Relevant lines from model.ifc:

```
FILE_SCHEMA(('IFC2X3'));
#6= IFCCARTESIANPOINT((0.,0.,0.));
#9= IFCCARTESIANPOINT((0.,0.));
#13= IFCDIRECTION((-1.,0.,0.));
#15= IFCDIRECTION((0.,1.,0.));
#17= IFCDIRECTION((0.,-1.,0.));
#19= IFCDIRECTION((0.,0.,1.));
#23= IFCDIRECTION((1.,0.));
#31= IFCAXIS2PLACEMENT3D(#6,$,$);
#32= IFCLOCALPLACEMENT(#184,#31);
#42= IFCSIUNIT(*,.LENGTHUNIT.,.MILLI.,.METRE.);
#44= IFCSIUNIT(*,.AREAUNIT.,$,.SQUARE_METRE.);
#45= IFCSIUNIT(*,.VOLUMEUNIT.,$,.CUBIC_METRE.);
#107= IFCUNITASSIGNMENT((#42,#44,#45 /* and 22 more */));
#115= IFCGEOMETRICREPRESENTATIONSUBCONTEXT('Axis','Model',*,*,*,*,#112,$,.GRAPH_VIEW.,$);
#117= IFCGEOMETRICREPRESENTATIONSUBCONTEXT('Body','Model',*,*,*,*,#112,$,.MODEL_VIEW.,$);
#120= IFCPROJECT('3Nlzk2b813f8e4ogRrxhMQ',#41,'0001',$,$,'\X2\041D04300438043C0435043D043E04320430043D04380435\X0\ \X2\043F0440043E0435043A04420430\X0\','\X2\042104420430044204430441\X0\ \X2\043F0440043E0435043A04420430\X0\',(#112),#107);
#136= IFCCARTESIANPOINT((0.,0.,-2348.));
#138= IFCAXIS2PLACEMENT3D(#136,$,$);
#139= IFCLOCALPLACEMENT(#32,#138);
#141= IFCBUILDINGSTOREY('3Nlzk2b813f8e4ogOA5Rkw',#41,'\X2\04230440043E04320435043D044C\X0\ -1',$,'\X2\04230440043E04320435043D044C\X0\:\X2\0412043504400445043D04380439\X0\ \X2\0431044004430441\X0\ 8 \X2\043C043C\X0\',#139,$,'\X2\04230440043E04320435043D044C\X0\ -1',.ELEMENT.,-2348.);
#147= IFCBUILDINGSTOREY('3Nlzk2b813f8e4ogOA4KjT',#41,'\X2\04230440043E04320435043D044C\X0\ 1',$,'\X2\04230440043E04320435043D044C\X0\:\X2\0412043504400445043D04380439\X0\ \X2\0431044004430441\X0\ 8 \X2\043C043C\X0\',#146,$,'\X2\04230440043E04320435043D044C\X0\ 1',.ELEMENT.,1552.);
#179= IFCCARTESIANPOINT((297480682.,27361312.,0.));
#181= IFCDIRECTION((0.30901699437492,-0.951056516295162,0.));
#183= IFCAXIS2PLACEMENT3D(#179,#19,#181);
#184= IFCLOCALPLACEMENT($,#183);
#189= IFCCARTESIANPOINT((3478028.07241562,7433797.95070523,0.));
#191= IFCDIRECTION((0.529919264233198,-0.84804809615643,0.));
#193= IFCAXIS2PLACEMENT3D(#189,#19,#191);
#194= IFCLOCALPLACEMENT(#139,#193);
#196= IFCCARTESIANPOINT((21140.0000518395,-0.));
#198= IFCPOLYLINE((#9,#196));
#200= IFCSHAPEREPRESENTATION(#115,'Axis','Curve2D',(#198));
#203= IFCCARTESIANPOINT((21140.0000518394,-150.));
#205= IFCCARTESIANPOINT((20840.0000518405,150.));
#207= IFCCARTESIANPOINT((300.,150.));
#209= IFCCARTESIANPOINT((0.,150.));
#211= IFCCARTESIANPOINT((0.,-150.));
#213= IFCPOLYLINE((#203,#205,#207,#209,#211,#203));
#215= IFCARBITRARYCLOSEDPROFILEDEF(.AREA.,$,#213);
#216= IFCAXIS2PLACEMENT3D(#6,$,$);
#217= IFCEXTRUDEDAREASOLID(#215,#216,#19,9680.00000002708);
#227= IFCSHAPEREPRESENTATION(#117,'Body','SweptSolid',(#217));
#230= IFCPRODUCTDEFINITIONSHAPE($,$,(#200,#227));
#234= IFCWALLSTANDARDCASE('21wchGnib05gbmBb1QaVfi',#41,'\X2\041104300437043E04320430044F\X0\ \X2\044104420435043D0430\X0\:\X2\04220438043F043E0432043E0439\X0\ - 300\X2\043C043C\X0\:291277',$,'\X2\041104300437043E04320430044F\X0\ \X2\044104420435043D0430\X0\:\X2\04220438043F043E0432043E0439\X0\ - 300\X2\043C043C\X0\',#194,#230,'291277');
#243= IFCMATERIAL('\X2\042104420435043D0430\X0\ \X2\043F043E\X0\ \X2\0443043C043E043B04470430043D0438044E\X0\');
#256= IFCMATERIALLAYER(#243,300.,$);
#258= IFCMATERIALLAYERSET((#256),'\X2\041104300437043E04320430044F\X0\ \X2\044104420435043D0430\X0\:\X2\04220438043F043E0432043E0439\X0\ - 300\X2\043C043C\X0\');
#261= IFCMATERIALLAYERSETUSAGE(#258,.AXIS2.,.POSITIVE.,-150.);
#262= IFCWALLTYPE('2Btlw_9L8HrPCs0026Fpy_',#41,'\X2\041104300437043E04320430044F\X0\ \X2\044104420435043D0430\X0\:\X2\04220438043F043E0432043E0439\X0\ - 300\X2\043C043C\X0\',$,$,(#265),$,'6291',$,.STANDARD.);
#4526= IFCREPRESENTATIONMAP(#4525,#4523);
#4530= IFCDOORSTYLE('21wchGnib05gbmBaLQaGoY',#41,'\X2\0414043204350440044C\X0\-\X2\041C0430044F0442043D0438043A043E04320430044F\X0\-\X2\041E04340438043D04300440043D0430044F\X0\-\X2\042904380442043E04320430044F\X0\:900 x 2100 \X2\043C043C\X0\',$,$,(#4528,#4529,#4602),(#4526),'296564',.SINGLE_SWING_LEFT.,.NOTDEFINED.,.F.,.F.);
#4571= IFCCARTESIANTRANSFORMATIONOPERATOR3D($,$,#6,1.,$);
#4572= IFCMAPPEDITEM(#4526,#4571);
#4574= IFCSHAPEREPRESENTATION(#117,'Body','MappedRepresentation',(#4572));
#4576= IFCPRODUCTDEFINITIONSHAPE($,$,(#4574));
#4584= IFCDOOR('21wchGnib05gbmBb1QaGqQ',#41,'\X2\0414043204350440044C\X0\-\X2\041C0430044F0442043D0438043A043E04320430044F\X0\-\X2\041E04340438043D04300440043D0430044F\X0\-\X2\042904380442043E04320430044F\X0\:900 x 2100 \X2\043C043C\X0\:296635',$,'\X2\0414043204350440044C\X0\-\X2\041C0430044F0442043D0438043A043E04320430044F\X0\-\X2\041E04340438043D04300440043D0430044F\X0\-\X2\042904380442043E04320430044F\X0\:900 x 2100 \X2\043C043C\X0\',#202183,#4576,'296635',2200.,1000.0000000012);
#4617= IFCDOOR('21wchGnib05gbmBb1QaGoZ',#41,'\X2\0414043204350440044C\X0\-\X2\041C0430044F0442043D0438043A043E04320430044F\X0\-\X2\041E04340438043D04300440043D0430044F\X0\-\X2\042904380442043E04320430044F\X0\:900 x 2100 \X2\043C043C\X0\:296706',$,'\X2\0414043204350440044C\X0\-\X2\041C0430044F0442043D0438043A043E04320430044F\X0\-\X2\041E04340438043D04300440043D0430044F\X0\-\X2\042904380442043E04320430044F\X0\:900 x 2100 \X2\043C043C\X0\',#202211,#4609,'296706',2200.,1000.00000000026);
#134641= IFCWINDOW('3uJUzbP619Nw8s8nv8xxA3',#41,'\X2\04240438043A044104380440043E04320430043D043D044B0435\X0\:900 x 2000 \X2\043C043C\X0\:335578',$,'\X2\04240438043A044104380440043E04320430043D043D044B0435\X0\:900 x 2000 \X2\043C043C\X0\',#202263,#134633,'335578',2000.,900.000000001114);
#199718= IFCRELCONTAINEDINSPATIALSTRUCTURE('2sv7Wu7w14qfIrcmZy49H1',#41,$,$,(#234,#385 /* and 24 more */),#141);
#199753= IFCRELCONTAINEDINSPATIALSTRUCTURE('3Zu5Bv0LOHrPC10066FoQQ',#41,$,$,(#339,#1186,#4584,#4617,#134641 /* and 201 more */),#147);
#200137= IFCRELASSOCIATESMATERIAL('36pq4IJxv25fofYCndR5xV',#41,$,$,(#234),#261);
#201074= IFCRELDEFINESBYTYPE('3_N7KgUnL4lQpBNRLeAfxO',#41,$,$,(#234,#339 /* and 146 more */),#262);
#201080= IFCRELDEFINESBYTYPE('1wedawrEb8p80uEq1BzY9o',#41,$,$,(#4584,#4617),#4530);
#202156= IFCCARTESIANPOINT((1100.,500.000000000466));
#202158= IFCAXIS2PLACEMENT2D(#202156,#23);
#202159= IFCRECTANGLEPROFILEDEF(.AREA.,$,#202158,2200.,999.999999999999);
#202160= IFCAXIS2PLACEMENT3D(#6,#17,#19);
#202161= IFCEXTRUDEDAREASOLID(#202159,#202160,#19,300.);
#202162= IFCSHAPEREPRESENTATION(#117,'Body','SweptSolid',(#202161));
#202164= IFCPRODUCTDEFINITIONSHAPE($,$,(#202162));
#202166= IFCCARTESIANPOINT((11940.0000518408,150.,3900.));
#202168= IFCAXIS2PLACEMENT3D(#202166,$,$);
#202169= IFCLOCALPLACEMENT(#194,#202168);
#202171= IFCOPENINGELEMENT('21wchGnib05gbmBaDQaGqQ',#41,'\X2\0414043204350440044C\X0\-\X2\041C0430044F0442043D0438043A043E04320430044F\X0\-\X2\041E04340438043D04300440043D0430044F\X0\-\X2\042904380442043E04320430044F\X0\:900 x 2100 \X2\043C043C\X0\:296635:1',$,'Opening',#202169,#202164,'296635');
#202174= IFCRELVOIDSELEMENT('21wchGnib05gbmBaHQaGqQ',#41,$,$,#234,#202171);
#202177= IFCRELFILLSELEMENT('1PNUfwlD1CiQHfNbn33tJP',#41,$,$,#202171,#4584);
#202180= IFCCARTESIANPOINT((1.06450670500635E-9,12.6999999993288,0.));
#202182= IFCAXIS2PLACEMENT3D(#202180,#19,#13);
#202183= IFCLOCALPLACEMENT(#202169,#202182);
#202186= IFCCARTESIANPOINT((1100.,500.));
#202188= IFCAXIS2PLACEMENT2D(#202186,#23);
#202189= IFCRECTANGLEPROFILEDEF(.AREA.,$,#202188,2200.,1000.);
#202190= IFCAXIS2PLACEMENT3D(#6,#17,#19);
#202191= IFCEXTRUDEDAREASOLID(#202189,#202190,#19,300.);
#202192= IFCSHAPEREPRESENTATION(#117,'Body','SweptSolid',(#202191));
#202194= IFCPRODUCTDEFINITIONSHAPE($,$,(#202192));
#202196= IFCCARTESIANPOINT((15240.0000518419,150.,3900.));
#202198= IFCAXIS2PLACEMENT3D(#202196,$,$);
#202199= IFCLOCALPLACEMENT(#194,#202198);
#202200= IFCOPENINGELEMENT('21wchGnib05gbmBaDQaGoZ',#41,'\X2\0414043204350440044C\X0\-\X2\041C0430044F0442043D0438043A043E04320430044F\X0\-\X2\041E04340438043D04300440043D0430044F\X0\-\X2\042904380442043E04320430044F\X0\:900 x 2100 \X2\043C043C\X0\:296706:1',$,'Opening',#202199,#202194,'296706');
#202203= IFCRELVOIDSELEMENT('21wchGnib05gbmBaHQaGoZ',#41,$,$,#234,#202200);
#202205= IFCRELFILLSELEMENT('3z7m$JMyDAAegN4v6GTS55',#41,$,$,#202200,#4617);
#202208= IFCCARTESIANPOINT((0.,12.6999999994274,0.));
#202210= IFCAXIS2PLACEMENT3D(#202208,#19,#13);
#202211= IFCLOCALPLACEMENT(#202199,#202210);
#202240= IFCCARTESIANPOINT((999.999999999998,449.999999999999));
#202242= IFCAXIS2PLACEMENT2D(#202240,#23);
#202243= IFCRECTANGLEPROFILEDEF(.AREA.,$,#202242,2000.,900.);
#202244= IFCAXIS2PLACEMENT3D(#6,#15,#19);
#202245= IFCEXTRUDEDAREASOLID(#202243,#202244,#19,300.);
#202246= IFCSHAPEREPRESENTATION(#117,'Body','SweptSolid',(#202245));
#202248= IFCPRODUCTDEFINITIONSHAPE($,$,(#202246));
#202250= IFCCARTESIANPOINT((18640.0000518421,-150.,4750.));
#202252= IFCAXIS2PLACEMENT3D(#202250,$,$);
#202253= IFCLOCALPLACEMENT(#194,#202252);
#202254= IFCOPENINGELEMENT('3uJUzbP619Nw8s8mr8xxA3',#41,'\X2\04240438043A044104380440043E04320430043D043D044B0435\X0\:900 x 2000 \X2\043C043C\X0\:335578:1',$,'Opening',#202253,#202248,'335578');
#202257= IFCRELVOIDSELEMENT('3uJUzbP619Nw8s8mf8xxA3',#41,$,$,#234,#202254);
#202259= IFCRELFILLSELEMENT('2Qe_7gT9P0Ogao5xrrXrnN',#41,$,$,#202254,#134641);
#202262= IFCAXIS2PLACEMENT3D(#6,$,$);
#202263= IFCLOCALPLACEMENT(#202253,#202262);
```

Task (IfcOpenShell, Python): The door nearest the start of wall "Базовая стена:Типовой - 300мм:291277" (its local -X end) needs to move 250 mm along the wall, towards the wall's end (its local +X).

```python
import ifcopenshell
import ifcopenshell.api.geometry
import ifcopenshell.util.placement
import ifcopenshell.util.unit

model = ifcopenshell.open("model.ifc")
unit_scale = ifcopenshell.util.unit.calculate_unit_scale(model)

door = model.by_id(4584)
opening = door.FillsVoids[0].RelatingOpeningElement
wall = opening.VoidsElements[0].RelatingBuildingElement

wall_matrix = ifcopenshell.util.placement.get_local_placement(wall.ObjectPlacement)
shift = wall_matrix[:3, 0] * 0.25 / unit_scale
before = ifcopenshell.util.placement.get_local_placement(door.ObjectPlacement)[:3, 3].copy()

# The door is placed relative to its opening, so it follows when the opening moves.
matrix = ifcopenshell.util.placement.get_local_placement(opening.ObjectPlacement)
matrix[:3, 3] += shift
ifcopenshell.api.geometry.edit_object_placement(
    model, product=opening, matrix=matrix, is_si=False, should_transform_children=True
)

after = ifcopenshell.util.placement.get_local_placement(door.ObjectPlacement)[:3, 3]
print("door moved by", (after - before).round(3) + 0.0)

model.write("model-out.ifc")
```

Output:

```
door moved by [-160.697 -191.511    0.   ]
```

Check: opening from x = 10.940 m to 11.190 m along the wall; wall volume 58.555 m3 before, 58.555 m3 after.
